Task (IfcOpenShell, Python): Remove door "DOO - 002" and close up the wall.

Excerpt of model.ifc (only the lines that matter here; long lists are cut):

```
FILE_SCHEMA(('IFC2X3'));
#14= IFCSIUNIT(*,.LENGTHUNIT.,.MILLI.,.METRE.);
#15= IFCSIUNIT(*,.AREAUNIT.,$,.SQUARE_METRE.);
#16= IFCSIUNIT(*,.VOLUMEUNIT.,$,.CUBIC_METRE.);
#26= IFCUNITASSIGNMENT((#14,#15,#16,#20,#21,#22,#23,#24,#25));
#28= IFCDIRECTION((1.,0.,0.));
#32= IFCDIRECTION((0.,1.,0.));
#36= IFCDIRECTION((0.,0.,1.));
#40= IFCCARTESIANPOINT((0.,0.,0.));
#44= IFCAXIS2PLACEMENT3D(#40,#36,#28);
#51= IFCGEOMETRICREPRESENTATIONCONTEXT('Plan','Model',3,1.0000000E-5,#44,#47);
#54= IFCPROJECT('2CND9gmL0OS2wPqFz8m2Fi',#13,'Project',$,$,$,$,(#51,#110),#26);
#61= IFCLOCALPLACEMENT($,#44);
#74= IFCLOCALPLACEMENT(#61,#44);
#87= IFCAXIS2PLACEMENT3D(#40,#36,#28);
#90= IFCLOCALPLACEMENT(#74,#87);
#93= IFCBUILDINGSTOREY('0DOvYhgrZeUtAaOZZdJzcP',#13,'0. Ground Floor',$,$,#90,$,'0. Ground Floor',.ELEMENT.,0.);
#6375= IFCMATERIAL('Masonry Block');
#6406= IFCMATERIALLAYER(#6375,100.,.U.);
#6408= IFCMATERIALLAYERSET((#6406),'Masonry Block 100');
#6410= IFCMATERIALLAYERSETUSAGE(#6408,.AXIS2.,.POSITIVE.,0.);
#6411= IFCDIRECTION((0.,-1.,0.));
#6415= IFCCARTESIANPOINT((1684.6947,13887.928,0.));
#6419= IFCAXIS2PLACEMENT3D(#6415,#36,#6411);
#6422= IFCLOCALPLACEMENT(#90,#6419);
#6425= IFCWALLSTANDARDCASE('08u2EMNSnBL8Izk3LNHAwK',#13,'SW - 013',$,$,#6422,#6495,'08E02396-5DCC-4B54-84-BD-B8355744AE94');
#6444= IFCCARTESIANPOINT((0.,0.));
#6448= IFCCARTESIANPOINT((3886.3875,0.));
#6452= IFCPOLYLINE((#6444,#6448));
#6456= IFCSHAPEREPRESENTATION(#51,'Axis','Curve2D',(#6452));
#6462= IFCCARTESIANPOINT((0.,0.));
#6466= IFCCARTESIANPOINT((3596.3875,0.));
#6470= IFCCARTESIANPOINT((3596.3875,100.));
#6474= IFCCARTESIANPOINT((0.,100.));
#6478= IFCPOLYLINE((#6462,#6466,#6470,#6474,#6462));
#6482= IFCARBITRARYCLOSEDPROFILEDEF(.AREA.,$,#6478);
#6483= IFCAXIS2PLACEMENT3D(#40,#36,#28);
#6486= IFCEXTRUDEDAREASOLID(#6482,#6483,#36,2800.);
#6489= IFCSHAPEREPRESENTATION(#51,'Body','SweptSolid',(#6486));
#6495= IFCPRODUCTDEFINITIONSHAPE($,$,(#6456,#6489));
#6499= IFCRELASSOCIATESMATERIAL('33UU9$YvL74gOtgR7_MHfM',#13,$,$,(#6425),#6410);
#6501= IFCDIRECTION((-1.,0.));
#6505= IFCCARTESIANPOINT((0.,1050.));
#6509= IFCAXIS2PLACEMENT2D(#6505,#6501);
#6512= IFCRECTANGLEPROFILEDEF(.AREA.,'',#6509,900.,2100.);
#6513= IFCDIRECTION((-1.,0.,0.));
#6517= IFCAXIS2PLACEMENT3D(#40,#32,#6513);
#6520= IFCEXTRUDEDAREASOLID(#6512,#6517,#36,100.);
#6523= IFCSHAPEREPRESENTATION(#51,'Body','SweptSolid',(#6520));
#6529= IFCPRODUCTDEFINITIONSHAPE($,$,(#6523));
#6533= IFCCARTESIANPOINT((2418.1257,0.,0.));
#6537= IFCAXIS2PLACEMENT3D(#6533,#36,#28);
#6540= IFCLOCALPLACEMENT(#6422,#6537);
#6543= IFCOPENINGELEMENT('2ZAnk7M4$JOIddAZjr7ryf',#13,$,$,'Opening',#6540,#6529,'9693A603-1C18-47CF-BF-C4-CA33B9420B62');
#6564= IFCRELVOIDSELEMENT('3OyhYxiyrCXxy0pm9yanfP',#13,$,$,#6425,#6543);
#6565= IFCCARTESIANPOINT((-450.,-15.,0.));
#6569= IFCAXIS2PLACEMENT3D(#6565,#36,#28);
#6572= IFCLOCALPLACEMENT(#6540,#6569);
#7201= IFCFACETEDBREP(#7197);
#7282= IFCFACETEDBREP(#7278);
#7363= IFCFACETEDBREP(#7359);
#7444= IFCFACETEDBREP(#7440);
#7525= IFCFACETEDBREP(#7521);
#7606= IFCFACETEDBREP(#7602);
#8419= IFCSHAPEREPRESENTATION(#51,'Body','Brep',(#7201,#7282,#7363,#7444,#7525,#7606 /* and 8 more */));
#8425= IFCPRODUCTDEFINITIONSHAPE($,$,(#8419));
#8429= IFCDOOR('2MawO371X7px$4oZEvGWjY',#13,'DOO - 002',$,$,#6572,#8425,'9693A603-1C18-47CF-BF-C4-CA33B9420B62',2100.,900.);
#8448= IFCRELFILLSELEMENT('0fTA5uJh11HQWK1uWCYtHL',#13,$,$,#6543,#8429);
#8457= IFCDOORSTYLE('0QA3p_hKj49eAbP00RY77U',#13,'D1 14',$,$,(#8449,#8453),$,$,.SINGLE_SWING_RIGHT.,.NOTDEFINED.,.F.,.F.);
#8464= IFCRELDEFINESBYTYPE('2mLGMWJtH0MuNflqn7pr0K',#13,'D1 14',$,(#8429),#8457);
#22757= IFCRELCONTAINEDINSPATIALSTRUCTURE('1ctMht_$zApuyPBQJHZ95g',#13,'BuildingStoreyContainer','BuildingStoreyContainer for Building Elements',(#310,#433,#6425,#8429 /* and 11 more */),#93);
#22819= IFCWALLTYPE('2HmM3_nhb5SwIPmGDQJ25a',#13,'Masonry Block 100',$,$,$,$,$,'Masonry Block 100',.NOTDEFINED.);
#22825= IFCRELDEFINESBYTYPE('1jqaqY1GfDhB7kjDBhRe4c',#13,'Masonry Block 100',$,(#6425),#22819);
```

```python
import ifcopenshell
import ifcopenshell.api.feature
import ifcopenshell.api.root
import ifcopenshell.geom
import ifcopenshell.util.shape

model = ifcopenshell.open("model.ifc")
settings = ifcopenshell.geom.settings()


def volume(element):
    """Net volume in cubic metres, openings subtracted."""
    shape = ifcopenshell.geom.create_shape(settings, element)
    return ifcopenshell.util.shape.get_volume(shape.geometry)


door = model.by_id(8429)
opening = door.FillsVoids[0].RelatingOpeningElement
wall = opening.VoidsElements[0].RelatingBuildingElement
before = volume(wall)

ifcopenshell.api.root.remove_product(model, product=door)
ifcopenshell.api.feature.remove_feature(model, feature=opening)

after = volume(wall)

print(f"wall volume {before:.3f} -> {after:.3f} m3")

model.write("model_v2.ifc")
```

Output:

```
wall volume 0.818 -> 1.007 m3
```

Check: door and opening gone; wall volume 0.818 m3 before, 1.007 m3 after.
